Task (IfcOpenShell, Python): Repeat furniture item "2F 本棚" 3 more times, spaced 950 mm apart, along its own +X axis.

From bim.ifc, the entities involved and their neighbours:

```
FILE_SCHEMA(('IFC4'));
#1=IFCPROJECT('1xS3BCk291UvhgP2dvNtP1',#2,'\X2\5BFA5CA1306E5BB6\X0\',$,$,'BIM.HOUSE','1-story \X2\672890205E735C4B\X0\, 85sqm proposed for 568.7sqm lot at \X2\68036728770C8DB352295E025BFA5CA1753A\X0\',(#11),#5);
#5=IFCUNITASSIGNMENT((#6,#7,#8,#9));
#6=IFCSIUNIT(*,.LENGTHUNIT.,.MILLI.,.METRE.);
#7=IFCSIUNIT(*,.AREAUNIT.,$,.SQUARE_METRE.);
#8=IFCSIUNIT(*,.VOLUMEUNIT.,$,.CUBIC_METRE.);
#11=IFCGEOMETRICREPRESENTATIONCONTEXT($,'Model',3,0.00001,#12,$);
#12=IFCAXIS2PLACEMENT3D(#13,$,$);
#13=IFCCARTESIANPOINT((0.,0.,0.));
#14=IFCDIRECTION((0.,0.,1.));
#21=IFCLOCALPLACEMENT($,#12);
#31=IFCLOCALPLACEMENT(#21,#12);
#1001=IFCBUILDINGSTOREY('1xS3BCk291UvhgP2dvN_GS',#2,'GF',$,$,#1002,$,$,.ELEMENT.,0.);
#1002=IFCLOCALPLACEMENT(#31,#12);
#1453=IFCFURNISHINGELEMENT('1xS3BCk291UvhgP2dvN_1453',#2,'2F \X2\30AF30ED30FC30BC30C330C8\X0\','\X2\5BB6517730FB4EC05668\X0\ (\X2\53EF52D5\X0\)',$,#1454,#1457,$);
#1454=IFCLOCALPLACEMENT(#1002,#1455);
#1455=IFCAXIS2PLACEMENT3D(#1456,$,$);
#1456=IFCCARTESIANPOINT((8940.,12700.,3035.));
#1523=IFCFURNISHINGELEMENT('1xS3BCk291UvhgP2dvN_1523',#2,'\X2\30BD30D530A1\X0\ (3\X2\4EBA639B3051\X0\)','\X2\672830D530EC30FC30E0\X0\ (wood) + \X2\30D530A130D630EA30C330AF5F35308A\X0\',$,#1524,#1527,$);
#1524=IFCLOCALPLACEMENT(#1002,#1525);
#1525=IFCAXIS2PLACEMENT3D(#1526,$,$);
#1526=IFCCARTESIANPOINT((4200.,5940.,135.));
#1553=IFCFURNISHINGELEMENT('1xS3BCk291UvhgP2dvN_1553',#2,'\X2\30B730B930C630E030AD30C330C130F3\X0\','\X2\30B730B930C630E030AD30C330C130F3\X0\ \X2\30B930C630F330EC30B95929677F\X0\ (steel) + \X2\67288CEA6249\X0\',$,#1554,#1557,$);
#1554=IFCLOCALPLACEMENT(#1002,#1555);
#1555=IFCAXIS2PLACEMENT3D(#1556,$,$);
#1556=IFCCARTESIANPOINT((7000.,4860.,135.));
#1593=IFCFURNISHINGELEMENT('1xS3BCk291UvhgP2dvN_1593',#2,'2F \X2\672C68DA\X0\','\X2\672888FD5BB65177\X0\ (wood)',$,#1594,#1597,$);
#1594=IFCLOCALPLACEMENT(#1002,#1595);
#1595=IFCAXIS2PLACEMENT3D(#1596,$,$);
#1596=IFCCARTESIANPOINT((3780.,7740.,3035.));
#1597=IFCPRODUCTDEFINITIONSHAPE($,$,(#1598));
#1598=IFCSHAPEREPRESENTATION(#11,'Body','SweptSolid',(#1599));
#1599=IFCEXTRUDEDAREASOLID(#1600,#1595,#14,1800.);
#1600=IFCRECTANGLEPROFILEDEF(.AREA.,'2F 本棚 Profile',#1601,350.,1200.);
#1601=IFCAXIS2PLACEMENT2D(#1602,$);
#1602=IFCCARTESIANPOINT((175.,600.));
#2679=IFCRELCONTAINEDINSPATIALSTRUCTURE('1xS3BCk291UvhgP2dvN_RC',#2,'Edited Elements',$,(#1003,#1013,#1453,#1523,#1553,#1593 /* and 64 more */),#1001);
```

```python
import ifcopenshell
import ifcopenshell.api.geometry
import ifcopenshell.api.root
import ifcopenshell.util.element
import ifcopenshell.util.placement

model = ifcopenshell.open("bim.ifc")


def reuse_history(source, copy):
    """copy_class also copies each property set's owner history, people and application; keep the originals."""
    for rel in copy.IsDefinedBy:
        if rel.is_a("IfcRelDefinesByProperties") and (history := rel.RelatingPropertyDefinition.OwnerHistory):
            rel.RelatingPropertyDefinition.OwnerHistory = source.OwnerHistory
            ifcopenshell.util.element.remove_deep2(model, history)


source = model.by_id(1593)
base = ifcopenshell.util.placement.get_local_placement(source.ObjectPlacement)
step = base[:3, 0] * 950.0

for i in range(1, 4):
    copy = ifcopenshell.api.root.copy_class(model, product=source)
    copy.Representation = ifcopenshell.util.element.copy_deep(
        model, source.Representation, exclude=["IfcGeometricRepresentationContext", "IfcRepresentationMap"]
    )
    reuse_history(source, copy)
    matrix = base.copy()
    matrix[:3, 3] += i * step
    print("added at", matrix[:3, 3].round(3) + 0.0)
    ifcopenshell.api.geometry.edit_object_placement(model, product=copy, matrix=matrix, is_si=False)

model.write("bim_updated.ifc")
```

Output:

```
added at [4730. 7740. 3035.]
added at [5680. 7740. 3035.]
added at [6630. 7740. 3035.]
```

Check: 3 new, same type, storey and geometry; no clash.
